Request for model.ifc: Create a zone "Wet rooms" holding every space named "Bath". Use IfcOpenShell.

First a look at what the model holds.

```python
import ifcopenshell

model = ifcopenshell.open("model.ifc")
print(model.schema)
seen = {}
for space in model.by_type("IfcSpace"):
    seen[space.LongName] = seen.get(space.LongName, 0) + 1
for name, count in sorted(seen.items(), key=str):
    print(count, "x", name)
print("zones:", [z.Name for z in model.by_type("IfcZone")][:20])
```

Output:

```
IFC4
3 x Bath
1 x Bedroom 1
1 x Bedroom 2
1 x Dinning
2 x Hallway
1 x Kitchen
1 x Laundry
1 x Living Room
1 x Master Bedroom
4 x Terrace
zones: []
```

```python
import ifcopenshell
import ifcopenshell.api.group
import ifcopenshell.api.root

model = ifcopenshell.open("model.ifc")

names = {"Bath"}
spaces = [s for s in model.by_type("IfcSpace") if s.LongName in names]

zone = ifcopenshell.api.root.create_entity(model, ifc_class="IfcZone", name="Wet rooms")
ifcopenshell.api.group.assign_group(model, products=spaces, group=zone)
print(len(spaces), "spaces in", zone.Name)

model.write("model-out.ifc")
```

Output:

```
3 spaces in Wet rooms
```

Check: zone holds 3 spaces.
